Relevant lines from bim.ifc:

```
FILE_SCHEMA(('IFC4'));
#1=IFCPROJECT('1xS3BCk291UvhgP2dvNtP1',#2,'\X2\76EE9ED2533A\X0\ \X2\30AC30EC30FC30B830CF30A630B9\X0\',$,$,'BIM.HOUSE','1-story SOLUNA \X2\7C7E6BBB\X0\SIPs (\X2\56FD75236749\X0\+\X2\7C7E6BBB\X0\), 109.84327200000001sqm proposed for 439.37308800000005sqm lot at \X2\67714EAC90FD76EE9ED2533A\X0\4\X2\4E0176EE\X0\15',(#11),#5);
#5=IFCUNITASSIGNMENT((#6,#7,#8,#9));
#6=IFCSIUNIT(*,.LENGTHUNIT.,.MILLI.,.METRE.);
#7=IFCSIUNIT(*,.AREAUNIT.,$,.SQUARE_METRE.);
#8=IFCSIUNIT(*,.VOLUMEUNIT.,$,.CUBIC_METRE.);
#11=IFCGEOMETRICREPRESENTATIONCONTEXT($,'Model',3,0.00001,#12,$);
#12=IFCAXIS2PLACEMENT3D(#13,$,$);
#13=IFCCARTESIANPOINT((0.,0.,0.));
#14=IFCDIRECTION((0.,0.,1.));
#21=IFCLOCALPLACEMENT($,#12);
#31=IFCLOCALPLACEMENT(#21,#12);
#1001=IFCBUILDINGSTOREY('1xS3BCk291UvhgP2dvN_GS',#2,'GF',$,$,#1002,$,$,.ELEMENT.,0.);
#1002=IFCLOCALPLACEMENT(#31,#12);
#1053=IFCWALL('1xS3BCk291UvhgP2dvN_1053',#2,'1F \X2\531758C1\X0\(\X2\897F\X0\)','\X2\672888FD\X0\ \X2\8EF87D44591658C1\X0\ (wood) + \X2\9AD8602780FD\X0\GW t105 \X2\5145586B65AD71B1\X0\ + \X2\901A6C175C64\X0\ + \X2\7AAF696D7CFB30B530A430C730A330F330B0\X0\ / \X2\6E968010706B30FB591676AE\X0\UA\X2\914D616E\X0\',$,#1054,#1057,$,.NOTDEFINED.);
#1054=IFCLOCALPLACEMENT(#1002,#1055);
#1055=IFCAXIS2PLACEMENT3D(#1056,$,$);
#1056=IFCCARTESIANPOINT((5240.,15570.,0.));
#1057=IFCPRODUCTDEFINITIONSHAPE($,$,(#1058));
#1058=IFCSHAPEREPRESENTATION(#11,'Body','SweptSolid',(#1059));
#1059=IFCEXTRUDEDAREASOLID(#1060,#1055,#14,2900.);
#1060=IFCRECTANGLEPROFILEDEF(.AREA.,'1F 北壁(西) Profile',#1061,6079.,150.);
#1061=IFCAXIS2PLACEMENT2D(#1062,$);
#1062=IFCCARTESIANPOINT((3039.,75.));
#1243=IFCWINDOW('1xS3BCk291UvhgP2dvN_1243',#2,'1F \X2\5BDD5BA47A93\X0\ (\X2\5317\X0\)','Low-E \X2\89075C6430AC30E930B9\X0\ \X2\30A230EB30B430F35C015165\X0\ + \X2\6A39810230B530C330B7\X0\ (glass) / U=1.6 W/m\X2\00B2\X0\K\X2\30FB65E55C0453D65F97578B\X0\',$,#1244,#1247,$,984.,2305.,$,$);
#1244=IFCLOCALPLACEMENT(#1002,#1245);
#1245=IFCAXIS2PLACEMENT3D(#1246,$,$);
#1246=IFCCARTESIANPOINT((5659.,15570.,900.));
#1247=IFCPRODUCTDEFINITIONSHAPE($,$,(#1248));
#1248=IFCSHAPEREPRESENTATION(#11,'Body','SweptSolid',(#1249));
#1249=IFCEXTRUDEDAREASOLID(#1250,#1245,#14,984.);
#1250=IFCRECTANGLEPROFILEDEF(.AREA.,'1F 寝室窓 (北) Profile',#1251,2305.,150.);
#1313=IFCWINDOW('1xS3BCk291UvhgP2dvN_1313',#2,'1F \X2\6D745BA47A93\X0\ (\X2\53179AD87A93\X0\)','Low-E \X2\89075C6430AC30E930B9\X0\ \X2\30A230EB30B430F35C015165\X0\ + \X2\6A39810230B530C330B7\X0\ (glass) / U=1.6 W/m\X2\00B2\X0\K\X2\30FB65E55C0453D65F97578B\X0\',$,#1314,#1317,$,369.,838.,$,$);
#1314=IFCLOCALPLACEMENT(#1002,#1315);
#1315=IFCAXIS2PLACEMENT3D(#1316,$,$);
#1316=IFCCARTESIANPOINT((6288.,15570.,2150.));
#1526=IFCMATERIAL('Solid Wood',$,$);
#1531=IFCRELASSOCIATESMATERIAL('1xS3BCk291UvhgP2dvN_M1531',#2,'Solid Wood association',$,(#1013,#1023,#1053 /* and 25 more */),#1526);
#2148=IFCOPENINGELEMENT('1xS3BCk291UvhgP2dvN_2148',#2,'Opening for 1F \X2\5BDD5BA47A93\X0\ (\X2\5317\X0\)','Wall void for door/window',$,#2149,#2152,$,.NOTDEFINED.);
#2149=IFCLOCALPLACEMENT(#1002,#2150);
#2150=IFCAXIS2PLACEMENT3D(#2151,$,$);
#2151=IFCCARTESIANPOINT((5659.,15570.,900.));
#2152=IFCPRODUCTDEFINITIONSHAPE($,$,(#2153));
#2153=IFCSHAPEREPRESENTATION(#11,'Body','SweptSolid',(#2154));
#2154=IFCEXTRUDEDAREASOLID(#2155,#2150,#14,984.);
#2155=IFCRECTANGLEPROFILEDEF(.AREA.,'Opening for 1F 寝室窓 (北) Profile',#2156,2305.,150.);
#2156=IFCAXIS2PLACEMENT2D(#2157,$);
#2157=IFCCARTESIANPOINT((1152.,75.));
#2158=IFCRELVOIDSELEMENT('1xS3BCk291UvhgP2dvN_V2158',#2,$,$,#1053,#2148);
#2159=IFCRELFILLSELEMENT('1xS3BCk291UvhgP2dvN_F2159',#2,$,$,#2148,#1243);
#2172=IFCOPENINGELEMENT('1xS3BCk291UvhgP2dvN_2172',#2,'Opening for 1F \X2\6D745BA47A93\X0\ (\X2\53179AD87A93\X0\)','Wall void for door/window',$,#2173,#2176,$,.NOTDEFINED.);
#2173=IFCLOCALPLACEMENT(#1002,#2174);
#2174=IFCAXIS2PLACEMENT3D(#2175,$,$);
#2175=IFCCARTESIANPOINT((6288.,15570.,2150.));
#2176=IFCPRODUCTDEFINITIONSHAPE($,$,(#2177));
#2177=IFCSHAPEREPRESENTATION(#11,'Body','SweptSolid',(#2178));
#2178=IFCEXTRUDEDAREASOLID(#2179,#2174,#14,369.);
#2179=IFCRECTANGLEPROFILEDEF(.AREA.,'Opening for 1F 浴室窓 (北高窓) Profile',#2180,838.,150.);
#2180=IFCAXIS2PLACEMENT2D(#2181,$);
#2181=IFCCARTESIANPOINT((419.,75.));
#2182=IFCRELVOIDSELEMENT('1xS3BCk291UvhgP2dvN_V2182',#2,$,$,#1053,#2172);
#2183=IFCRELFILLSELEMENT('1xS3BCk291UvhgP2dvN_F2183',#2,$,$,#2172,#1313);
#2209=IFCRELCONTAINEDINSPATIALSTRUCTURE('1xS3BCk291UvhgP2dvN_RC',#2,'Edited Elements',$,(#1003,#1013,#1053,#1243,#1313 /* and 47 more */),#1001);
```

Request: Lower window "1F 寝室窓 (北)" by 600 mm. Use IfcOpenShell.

```python
import numpy as np
import ifcopenshell
import ifcopenshell.api.geometry
import ifcopenshell.util.placement
import ifcopenshell.util.unit

model = ifcopenshell.open("bim.ifc")
unit_scale = ifcopenshell.util.unit.calculate_unit_scale(model)

window = model.by_guid("1xS3BCk291UvhgP2dvN_1243")
opening = window.FillsVoids[0].RelatingOpeningElement
dz = -600.0

shift = np.array([0.0, 0.0, dz])
# The window is not placed relative to its opening, so move both.
for product in (opening, window):
    matrix = ifcopenshell.util.placement.get_local_placement(product.ObjectPlacement)
    matrix[:3, 3] += shift
    ifcopenshell.api.geometry.edit_object_placement(model, product=product, matrix=matrix, is_si=False)

print(f"moved by {dz * unit_scale:+.3f} m")

model.write("bim-out.ifc")
```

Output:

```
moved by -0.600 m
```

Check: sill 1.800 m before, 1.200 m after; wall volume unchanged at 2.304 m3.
